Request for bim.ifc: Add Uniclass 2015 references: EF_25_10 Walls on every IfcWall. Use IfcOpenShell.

First a look at what the model holds.

```python
import ifcopenshell

model = ifcopenshell.open("bim.ifc")
print(model.schema)
print("classifications:", [c.Name for c in model.by_type("IfcClassification")])
for ifc_class in ("IfcDoor", "IfcRoof", "IfcStair", "IfcWall", "IfcWindow"):
    print(ifc_class, len(model.by_type(ifc_class)))
```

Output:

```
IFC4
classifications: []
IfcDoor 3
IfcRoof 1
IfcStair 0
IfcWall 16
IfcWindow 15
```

```python
import ifcopenshell
import ifcopenshell.api.classification

model = ifcopenshell.open("bim.ifc")

system = ifcopenshell.api.classification.add_classification(model, classification="Uniclass 2015")

codes = {
    "IfcWall": ("EF_25_10", "Walls"),
}
for ifc_class, (code, name) in codes.items():
    products = model.by_type(ifc_class)
    ifcopenshell.api.classification.add_reference(
        model, products=products, classification=system, identification=code, name=name
    )
    print(code, len(products))

model.write("bim_edited.ifc")
```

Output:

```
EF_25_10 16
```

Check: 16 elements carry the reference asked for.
